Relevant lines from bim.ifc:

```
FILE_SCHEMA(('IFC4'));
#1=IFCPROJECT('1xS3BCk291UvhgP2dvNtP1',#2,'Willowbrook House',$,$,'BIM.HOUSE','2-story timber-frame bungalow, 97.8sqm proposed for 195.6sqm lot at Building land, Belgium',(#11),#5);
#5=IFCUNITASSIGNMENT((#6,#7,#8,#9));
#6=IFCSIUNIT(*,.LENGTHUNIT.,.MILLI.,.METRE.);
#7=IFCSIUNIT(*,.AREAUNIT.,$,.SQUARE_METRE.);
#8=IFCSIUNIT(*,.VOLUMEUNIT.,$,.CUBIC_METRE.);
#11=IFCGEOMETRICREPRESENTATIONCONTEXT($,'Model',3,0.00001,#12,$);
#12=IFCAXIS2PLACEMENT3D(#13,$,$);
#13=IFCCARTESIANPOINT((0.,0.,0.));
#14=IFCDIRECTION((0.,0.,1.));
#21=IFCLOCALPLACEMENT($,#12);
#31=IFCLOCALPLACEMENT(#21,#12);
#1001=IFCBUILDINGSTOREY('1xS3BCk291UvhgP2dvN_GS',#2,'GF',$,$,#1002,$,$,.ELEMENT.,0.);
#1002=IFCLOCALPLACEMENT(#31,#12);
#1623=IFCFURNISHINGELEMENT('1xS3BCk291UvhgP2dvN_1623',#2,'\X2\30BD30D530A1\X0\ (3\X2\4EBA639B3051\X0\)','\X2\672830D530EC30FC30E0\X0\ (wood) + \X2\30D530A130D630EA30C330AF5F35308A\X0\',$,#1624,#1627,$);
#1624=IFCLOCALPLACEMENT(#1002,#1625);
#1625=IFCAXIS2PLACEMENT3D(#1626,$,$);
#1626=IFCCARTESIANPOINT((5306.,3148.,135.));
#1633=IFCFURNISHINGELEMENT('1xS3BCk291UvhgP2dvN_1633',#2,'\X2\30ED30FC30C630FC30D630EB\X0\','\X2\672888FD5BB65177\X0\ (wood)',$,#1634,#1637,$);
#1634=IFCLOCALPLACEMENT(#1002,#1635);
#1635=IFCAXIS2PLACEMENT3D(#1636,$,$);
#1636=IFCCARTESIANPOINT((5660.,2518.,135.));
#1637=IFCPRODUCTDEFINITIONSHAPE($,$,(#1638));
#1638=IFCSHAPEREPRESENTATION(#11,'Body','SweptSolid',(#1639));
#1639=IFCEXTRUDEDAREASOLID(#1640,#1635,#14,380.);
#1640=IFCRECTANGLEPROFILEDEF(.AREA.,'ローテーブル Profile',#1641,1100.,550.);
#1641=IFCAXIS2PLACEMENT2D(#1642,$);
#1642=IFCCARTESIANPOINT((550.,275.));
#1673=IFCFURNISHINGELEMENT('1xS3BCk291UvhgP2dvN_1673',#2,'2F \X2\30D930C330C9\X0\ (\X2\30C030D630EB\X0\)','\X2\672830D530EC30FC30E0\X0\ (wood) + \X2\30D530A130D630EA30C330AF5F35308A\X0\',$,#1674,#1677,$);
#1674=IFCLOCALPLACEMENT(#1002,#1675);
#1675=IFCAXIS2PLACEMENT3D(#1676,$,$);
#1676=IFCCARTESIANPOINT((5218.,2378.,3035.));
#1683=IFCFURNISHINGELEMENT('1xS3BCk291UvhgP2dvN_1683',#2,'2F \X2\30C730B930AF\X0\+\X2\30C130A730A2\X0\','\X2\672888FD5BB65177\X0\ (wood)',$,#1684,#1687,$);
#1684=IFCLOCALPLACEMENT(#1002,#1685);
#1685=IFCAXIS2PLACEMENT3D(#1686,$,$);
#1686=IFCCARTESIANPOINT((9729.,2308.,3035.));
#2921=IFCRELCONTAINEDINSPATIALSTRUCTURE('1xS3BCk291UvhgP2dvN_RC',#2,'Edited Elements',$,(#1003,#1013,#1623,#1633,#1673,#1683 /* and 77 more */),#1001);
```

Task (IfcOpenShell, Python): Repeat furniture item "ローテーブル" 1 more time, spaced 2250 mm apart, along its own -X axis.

```python
import ifcopenshell
import ifcopenshell.api.geometry
import ifcopenshell.api.root
import ifcopenshell.util.element
import ifcopenshell.util.placement
import ifcopenshell.util.unit

model = ifcopenshell.open("bim.ifc")
unit_scale = ifcopenshell.util.unit.calculate_unit_scale(model)


def reuse_history(source, copy):
    """copy_class also copies each property set's owner history, people and application; keep the originals."""
    for rel in copy.IsDefinedBy:
        if rel.is_a("IfcRelDefinesByProperties") and (history := rel.RelatingPropertyDefinition.OwnerHistory):
            rel.RelatingPropertyDefinition.OwnerHistory = source.OwnerHistory
            ifcopenshell.util.element.remove_deep2(model, history)


source = model.by_guid("1xS3BCk291UvhgP2dvN_1633")
base = ifcopenshell.util.placement.get_local_placement(source.ObjectPlacement)
step = -base[:3, 0] * 2.25 / unit_scale

for i in range(1, 2):
    copy = ifcopenshell.api.root.copy_class(model, product=source)
    copy.Representation = ifcopenshell.util.element.copy_deep(
        model, source.Representation, exclude=["IfcGeometricRepresentationContext", "IfcRepresentationMap"]
    )
    reuse_history(source, copy)
    matrix = base.copy()
    matrix[:3, 3] += i * step
    print("added at", matrix[:3, 3].round(3) + 0.0)
    ifcopenshell.api.geometry.edit_object_placement(model, product=copy, matrix=matrix, is_si=False)

model.write("bim-out.ifc")
```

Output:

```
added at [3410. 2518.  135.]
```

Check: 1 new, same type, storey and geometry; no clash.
